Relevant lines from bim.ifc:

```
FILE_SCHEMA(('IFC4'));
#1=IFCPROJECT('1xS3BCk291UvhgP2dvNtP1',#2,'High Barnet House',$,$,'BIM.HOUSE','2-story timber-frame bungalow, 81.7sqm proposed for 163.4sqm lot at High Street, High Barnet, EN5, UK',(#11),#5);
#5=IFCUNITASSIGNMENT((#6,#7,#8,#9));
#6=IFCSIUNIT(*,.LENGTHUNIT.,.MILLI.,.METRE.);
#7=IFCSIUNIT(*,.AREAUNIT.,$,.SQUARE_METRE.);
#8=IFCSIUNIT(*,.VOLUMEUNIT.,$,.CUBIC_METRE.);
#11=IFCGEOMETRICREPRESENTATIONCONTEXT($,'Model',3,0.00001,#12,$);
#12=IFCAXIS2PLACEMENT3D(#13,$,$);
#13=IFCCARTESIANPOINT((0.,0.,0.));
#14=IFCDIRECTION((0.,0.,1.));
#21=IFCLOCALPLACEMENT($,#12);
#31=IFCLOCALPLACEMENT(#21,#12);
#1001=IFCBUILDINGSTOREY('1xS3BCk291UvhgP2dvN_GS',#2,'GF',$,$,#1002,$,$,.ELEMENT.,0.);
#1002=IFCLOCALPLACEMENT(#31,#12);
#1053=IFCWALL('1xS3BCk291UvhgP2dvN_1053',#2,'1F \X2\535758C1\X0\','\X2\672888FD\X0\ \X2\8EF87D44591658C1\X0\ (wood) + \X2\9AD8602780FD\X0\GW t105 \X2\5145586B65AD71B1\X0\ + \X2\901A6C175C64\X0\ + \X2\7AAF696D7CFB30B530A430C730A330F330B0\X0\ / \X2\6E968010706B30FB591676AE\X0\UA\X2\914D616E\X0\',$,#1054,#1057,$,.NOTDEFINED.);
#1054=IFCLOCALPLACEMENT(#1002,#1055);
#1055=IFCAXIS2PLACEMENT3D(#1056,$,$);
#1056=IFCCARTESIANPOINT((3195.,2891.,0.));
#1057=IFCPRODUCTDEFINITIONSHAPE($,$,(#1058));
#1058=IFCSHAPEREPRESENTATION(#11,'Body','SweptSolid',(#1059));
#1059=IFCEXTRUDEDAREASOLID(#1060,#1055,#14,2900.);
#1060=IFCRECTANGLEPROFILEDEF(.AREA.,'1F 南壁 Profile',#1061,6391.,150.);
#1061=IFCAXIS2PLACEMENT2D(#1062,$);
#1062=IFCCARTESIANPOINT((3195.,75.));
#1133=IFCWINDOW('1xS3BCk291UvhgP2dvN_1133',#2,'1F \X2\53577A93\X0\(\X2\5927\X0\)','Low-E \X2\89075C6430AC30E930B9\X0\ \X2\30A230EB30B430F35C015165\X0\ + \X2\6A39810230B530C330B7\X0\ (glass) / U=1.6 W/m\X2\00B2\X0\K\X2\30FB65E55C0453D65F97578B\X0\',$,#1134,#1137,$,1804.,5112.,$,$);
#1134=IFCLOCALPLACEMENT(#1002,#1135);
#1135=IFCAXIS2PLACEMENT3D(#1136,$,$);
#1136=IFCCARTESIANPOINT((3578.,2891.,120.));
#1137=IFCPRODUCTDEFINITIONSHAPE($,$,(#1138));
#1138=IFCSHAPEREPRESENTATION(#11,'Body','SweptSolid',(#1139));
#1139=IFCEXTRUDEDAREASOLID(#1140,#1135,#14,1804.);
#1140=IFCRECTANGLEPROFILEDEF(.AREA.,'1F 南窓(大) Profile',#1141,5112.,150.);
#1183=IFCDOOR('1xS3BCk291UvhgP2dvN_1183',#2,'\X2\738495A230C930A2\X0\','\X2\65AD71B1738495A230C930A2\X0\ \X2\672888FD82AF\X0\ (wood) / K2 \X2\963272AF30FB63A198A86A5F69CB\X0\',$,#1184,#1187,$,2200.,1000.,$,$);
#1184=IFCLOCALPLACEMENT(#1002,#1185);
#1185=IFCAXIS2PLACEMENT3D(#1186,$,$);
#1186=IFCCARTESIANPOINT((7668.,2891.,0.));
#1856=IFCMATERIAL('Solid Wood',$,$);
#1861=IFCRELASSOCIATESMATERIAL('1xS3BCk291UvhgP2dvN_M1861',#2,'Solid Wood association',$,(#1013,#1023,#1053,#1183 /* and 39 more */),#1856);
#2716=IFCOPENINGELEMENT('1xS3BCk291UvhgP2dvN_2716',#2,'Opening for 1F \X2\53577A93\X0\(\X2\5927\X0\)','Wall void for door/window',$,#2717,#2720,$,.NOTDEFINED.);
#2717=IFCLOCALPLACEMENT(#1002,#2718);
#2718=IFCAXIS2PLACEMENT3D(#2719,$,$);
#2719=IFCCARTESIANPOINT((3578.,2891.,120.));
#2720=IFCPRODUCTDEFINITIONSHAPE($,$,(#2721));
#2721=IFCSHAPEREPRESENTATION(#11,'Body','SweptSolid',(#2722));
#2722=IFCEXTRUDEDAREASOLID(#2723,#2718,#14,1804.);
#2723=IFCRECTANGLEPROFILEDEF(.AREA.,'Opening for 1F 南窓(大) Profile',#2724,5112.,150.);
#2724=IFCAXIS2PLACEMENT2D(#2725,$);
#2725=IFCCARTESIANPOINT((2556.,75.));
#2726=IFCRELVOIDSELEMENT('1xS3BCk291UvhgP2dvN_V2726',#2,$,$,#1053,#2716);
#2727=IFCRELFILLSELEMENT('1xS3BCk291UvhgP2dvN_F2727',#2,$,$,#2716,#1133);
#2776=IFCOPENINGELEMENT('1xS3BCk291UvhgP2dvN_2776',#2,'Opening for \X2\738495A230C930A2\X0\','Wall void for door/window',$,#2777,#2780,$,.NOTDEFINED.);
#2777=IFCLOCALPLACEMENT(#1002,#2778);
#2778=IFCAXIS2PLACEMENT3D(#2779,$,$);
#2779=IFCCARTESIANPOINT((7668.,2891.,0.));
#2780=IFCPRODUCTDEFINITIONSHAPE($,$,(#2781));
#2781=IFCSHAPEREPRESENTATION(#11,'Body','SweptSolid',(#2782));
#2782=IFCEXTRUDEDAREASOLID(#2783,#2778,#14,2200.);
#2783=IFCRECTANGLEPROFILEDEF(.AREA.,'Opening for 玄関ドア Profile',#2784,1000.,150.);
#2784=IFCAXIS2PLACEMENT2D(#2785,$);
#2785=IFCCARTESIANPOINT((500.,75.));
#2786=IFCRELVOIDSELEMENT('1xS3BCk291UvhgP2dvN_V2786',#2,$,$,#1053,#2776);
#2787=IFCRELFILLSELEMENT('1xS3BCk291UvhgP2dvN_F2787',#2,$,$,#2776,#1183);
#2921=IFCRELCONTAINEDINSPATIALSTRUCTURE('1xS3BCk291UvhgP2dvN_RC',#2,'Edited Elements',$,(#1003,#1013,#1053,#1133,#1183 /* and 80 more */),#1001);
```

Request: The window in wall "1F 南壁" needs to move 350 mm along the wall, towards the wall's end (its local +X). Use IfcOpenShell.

```python
import ifcopenshell
import ifcopenshell.api.geometry
import ifcopenshell.util.placement

model = ifcopenshell.open("bim.ifc")

window = model.by_id(1133)
opening = window.FillsVoids[0].RelatingOpeningElement
wall = opening.VoidsElements[0].RelatingBuildingElement

wall_matrix = ifcopenshell.util.placement.get_local_placement(wall.ObjectPlacement)
shift = wall_matrix[:3, 0] * 350.0
before = ifcopenshell.util.placement.get_local_placement(window.ObjectPlacement)[:3, 3].copy()

# The window is not placed relative to its opening, so move both.
for product in (opening, window):
    matrix = ifcopenshell.util.placement.get_local_placement(product.ObjectPlacement)
    matrix[:3, 3] += shift
    ifcopenshell.api.geometry.edit_object_placement(model, product=product, matrix=matrix, is_si=False)

after = ifcopenshell.util.placement.get_local_placement(window.ObjectPlacement)[:3, 3]
print("window moved by", (after - before).round(3) + 0.0)

model.write("bim_updated.ifc")
```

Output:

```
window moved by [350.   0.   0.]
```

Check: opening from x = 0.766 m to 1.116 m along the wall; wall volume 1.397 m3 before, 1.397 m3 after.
